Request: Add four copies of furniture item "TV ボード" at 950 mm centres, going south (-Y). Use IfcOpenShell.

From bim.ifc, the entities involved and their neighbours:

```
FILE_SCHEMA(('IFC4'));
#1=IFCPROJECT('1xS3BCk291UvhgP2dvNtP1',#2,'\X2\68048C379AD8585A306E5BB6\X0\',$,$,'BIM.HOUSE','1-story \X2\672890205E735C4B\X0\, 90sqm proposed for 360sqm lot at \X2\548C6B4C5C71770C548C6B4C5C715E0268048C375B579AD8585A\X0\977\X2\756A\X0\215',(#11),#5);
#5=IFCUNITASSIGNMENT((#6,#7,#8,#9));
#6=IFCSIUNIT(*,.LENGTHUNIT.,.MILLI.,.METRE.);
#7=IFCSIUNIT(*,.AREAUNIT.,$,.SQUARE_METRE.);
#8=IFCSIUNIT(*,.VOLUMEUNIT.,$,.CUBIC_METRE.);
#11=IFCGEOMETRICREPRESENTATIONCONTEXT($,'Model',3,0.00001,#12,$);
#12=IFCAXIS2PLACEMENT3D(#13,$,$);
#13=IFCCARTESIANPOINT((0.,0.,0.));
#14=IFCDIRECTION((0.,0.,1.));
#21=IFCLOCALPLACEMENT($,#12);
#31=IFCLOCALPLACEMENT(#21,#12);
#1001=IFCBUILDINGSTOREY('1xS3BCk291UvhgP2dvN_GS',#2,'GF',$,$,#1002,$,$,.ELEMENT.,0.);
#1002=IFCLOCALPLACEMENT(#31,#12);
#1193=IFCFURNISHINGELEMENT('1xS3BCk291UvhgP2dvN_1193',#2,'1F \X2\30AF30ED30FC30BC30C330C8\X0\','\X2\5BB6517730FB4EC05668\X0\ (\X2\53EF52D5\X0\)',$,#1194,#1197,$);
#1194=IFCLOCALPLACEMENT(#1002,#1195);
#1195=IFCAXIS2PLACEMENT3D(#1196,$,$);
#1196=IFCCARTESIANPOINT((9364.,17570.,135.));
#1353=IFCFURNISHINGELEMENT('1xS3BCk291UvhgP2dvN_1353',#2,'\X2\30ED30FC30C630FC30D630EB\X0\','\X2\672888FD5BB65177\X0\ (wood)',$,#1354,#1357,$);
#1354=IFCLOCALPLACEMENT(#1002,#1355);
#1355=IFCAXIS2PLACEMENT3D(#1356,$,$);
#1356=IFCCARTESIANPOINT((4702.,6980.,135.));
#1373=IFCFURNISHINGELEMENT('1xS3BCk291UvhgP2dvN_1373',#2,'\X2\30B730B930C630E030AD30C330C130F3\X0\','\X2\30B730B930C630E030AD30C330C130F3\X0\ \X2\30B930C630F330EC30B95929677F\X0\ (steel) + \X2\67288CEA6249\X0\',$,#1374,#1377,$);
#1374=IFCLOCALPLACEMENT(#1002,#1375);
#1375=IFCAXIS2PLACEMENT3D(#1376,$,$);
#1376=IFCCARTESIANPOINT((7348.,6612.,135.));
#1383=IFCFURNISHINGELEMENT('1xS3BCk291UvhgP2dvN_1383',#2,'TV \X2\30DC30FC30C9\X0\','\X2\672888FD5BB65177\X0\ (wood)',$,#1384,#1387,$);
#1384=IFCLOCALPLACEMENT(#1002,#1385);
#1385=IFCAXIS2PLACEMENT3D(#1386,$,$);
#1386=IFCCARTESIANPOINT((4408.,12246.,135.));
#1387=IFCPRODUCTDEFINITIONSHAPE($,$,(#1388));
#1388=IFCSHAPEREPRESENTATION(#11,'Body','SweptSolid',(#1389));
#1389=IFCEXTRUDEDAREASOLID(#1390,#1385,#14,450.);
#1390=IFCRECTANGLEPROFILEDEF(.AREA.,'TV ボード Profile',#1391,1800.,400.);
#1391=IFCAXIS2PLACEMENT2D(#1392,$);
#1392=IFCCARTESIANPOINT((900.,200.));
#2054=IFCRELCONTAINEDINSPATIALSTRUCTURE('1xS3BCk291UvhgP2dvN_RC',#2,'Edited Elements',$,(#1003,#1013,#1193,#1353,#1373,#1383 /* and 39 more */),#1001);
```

```python
import numpy as np
import ifcopenshell
import ifcopenshell.api.geometry
import ifcopenshell.api.root
import ifcopenshell.util.element
import ifcopenshell.util.placement
import ifcopenshell.util.unit

model = ifcopenshell.open("bim.ifc")
unit_scale = ifcopenshell.util.unit.calculate_unit_scale(model)


def reuse_history(source, copy):
    """copy_class also copies each property set's owner history, people and application; keep the originals."""
    for rel in copy.IsDefinedBy:
        if rel.is_a("IfcRelDefinesByProperties") and (history := rel.RelatingPropertyDefinition.OwnerHistory):
            rel.RelatingPropertyDefinition.OwnerHistory = source.OwnerHistory
            ifcopenshell.util.element.remove_deep2(model, history)


source = model.by_guid("1xS3BCk291UvhgP2dvN_1383")
base = ifcopenshell.util.placement.get_local_placement(source.ObjectPlacement)
step = np.array([0.0, -1.0, 0.0]) * 0.95 / unit_scale

for i in range(1, 5):
    copy = ifcopenshell.api.root.copy_class(model, product=source)
    copy.Representation = ifcopenshell.util.element.copy_deep(
        model, source.Representation, exclude=["IfcGeometricRepresentationContext", "IfcRepresentationMap"]
    )
    reuse_history(source, copy)
    matrix = base.copy()
    matrix[:3, 3] += i * step
    print("added at", matrix[:3, 3].round(3) + 0.0)
    ifcopenshell.api.geometry.edit_object_placement(model, product=copy, matrix=matrix, is_si=False)

model.write("bim_updated.ifc")
```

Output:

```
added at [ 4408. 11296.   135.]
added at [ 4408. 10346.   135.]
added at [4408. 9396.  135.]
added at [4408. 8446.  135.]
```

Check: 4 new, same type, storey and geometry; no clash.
